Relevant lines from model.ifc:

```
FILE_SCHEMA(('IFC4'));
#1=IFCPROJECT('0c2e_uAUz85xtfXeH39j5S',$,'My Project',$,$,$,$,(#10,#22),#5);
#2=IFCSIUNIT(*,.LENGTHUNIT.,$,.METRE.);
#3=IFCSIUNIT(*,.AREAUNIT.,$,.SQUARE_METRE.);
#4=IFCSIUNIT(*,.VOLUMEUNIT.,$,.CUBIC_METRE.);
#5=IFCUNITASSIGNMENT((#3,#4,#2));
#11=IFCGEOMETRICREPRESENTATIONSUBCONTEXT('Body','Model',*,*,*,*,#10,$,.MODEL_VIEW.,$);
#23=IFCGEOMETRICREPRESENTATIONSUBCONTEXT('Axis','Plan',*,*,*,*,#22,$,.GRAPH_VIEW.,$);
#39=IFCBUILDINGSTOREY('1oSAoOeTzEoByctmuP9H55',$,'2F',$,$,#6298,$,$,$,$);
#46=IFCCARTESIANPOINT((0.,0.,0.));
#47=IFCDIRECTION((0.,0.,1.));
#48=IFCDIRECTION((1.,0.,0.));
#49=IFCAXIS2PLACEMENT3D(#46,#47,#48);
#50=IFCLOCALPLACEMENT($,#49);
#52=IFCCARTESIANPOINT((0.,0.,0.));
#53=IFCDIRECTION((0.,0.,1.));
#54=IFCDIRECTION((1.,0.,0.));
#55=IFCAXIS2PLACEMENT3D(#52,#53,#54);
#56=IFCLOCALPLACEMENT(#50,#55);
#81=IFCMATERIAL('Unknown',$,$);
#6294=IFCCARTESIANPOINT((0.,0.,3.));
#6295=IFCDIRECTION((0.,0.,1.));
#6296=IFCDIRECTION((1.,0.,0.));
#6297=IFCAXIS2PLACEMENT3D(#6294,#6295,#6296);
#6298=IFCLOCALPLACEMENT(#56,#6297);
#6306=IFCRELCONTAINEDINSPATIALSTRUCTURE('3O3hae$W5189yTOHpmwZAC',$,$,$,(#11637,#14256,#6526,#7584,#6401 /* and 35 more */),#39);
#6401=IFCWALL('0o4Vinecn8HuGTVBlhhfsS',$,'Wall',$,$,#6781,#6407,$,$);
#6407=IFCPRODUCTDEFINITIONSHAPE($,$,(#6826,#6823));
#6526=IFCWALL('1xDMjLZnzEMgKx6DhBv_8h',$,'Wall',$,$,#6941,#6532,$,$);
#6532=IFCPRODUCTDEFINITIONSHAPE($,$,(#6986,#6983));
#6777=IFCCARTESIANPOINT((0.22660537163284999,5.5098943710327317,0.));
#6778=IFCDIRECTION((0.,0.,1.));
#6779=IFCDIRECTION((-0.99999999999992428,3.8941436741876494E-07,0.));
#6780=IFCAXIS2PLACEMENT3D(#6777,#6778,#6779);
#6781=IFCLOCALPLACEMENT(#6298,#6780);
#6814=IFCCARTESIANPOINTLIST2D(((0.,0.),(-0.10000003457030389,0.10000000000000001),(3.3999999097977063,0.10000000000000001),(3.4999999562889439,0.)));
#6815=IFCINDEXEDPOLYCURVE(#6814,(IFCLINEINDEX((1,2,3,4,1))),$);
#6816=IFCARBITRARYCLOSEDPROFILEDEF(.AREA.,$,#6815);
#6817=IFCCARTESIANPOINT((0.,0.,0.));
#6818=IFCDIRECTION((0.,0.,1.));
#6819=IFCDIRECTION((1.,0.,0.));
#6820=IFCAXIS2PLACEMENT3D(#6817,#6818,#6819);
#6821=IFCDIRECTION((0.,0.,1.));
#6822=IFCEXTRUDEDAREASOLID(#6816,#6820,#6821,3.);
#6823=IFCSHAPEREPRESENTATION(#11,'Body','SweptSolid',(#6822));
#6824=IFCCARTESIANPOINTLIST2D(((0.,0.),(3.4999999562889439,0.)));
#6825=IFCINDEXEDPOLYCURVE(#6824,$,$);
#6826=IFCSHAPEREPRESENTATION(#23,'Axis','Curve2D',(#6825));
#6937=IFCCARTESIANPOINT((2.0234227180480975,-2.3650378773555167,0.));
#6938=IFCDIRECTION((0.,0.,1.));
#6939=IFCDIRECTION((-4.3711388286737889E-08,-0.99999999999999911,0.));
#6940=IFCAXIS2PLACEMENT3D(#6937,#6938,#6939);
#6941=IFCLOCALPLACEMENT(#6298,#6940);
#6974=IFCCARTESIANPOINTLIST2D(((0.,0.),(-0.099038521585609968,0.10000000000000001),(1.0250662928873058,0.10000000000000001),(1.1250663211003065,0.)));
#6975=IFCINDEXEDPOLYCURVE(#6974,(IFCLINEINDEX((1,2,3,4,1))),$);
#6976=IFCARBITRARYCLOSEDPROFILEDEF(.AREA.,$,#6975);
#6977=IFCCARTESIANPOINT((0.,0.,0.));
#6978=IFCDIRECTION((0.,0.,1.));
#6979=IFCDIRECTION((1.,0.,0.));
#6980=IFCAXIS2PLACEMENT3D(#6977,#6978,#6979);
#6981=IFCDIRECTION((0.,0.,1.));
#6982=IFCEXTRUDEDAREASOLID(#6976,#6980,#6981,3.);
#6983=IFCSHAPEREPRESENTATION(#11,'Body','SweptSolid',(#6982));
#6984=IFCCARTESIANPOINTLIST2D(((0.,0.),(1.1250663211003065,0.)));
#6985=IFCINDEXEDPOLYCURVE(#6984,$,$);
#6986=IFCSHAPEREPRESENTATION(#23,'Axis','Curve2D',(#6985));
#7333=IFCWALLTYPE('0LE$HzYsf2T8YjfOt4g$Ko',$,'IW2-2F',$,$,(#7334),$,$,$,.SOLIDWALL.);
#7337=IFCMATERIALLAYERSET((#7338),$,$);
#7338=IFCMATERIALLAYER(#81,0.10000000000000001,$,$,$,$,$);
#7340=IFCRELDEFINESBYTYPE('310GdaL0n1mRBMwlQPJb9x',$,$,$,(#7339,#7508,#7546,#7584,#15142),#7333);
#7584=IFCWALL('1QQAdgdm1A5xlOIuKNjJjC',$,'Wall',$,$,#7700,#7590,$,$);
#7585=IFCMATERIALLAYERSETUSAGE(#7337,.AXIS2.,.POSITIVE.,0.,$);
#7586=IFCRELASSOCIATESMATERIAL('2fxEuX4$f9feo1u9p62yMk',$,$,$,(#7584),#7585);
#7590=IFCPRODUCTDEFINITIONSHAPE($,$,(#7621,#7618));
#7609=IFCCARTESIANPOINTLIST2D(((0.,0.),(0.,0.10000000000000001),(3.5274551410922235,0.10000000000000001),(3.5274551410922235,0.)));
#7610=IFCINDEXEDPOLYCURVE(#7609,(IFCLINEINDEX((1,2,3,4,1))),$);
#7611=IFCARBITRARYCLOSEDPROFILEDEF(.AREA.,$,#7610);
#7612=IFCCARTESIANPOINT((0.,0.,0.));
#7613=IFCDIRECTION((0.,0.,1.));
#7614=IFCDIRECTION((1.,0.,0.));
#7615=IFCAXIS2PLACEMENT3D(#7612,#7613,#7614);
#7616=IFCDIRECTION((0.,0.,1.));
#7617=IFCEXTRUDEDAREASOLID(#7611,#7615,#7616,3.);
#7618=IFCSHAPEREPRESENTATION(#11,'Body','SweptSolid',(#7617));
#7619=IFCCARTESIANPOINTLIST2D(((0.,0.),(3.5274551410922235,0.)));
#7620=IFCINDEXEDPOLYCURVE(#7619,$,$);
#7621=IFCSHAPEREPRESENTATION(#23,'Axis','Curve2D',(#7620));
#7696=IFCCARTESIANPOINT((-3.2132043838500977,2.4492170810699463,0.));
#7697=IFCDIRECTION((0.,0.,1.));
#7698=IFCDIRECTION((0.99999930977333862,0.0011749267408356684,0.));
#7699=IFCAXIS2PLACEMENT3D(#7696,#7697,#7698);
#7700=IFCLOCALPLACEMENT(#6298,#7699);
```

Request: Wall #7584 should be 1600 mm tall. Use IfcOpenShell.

```python
import ifcopenshell
import ifcopenshell.geom
import ifcopenshell.util.representation
import ifcopenshell.util.shape
import ifcopenshell.util.unit

model = ifcopenshell.open("model.ifc")
unit_scale = ifcopenshell.util.unit.calculate_unit_scale(model)
settings = ifcopenshell.geom.settings()


def volume(element):
    """Net volume in cubic metres, openings subtracted."""
    shape = ifcopenshell.geom.create_shape(settings, element)
    return ifcopenshell.util.shape.get_volume(shape.geometry)


wall = model.by_guid("1QQAdgdm1A5xlOIuKNjJjC")
before = volume(wall)

body = ifcopenshell.util.representation.get_representation(wall, "Model", "Body")
solid = body.Items[0]
old_height = solid.Depth
solid.Depth = 1.6 / unit_scale
after = volume(wall)

print(f"height {old_height:g} -> {solid.Depth:g}, volume {before:.3f} -> {after:.3f} m3")

model.write("model_edited.ifc")
```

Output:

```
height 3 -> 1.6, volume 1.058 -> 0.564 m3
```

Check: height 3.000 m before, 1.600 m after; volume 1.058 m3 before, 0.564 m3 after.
